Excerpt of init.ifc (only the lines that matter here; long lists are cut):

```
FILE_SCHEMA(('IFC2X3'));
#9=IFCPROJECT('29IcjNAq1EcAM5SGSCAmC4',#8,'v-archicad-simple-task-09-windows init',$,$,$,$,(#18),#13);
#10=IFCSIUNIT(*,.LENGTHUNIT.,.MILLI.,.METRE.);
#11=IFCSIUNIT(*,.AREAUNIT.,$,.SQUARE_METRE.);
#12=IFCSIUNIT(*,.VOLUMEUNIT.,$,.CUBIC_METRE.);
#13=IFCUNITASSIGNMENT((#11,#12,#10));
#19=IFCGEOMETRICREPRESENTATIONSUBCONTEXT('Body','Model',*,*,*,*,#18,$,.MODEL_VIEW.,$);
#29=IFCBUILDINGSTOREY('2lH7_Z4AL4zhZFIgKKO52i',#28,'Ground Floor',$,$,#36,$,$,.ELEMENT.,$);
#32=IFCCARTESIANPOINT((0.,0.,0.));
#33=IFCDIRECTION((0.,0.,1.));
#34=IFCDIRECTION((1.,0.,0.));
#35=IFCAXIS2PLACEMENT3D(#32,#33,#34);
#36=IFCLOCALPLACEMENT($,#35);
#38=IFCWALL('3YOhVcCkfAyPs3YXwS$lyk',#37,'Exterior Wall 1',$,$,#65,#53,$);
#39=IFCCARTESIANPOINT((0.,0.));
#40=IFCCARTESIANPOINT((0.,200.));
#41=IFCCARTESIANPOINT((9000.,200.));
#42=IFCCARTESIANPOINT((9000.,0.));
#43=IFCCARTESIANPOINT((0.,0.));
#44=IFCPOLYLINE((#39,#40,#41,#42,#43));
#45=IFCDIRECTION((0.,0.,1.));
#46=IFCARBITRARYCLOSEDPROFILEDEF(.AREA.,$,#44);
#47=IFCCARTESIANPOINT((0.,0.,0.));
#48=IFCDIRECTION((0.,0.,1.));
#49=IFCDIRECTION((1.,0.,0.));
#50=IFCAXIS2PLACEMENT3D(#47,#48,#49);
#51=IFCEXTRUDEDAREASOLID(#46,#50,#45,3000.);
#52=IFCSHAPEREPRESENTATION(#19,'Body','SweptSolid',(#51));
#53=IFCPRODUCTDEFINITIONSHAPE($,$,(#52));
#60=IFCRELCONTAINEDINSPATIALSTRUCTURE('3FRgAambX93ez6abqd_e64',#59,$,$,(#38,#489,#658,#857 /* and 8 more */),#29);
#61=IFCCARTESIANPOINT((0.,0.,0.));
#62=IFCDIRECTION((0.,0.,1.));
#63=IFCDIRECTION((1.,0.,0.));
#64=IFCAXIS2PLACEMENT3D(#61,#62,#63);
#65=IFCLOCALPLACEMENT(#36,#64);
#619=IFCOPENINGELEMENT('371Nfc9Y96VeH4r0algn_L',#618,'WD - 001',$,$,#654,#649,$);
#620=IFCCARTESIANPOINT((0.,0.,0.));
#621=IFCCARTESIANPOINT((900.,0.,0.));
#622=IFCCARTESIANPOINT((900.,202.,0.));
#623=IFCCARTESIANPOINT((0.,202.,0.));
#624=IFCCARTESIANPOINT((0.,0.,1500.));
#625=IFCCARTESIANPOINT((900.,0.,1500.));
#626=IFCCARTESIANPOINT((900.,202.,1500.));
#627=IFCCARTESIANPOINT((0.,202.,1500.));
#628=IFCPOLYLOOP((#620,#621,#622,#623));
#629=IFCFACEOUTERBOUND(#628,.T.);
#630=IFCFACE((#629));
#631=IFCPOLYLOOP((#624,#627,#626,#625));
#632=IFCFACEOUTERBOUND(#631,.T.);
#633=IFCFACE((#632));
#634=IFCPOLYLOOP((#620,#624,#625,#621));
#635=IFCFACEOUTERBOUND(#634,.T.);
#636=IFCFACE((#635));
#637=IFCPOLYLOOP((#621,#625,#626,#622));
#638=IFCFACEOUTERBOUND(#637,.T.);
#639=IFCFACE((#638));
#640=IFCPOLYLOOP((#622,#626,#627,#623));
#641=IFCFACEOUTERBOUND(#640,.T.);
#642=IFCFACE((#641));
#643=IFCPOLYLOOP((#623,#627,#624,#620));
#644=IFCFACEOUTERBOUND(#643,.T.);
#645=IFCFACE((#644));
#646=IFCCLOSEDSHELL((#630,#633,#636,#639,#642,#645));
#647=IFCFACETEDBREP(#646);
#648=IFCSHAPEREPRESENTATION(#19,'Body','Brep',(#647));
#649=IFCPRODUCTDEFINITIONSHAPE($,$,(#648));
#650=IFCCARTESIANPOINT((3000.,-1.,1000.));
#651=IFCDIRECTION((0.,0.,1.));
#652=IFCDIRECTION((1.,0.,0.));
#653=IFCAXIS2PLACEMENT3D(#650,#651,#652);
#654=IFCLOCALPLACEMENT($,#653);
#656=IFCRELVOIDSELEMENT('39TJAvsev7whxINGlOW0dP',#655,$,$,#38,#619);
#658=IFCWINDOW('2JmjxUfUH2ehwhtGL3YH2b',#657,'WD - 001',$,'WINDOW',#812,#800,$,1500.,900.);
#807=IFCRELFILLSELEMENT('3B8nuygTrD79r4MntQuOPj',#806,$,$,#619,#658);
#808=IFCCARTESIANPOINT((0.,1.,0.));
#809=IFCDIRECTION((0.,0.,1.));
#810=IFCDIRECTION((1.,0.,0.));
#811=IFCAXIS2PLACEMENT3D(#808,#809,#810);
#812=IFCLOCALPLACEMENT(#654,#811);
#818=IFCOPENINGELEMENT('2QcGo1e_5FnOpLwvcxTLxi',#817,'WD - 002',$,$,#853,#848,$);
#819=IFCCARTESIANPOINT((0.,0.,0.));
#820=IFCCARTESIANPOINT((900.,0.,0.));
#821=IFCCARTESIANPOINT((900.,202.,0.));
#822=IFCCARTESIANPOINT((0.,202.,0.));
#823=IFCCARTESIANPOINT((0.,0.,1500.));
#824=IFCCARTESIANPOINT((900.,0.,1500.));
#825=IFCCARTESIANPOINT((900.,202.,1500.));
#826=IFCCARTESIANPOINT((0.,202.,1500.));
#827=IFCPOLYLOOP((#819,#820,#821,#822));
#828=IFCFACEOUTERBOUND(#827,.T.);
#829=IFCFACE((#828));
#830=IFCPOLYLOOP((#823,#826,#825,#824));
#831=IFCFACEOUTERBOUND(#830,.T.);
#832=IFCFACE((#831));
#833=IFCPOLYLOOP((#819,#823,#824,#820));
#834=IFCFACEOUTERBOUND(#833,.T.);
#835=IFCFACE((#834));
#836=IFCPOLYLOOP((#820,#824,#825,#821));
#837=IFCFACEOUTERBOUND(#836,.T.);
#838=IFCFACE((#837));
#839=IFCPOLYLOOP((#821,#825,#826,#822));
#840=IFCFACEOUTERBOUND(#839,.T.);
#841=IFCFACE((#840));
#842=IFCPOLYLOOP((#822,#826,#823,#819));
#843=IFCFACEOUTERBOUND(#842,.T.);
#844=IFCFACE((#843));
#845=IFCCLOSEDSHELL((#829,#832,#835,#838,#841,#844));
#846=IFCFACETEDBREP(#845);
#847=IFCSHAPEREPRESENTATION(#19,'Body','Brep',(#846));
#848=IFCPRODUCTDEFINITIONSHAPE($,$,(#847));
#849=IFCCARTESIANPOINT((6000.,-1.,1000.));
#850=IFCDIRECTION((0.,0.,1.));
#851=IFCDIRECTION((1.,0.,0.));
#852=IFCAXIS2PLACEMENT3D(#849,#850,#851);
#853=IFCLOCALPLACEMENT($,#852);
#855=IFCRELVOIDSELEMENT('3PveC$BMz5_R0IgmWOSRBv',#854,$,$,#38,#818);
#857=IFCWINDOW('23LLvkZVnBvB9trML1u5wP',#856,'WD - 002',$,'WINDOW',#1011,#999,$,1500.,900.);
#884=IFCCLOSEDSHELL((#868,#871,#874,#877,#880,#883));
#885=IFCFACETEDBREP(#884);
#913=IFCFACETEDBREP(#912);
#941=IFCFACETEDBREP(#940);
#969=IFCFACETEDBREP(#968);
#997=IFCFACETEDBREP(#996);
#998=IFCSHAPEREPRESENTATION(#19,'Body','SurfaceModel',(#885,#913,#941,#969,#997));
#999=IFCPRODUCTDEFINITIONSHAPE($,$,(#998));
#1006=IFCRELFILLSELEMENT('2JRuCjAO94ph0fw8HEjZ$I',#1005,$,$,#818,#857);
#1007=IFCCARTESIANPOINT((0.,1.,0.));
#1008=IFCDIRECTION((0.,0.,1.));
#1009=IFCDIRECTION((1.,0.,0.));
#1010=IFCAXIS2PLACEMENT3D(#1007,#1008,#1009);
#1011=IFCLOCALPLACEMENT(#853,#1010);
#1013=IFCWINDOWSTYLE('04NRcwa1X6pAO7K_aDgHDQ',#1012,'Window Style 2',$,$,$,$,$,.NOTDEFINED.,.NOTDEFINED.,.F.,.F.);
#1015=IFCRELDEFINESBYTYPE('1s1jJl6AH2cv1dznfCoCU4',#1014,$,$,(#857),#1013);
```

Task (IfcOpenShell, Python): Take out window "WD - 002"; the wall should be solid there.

```python
import ifcopenshell
import ifcopenshell.api.feature
import ifcopenshell.api.root
import ifcopenshell.geom
import ifcopenshell.util.shape

model = ifcopenshell.open("init.ifc")
settings = ifcopenshell.geom.settings()


def volume(element):
    """Net volume in cubic metres, openings subtracted."""
    shape = ifcopenshell.geom.create_shape(settings, element)
    return ifcopenshell.util.shape.get_volume(shape.geometry)


window = model.by_guid("23LLvkZVnBvB9trML1u5wP")
opening = window.FillsVoids[0].RelatingOpeningElement
wall = opening.VoidsElements[0].RelatingBuildingElement
before = volume(wall)

ifcopenshell.api.root.remove_product(model, product=window)
ifcopenshell.api.feature.remove_feature(model, feature=opening)

after = volume(wall)

print(f"wall volume {before:.3f} -> {after:.3f} m3")

model.write("init_v2.ifc")
```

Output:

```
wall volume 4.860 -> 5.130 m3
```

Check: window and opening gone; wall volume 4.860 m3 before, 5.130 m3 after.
